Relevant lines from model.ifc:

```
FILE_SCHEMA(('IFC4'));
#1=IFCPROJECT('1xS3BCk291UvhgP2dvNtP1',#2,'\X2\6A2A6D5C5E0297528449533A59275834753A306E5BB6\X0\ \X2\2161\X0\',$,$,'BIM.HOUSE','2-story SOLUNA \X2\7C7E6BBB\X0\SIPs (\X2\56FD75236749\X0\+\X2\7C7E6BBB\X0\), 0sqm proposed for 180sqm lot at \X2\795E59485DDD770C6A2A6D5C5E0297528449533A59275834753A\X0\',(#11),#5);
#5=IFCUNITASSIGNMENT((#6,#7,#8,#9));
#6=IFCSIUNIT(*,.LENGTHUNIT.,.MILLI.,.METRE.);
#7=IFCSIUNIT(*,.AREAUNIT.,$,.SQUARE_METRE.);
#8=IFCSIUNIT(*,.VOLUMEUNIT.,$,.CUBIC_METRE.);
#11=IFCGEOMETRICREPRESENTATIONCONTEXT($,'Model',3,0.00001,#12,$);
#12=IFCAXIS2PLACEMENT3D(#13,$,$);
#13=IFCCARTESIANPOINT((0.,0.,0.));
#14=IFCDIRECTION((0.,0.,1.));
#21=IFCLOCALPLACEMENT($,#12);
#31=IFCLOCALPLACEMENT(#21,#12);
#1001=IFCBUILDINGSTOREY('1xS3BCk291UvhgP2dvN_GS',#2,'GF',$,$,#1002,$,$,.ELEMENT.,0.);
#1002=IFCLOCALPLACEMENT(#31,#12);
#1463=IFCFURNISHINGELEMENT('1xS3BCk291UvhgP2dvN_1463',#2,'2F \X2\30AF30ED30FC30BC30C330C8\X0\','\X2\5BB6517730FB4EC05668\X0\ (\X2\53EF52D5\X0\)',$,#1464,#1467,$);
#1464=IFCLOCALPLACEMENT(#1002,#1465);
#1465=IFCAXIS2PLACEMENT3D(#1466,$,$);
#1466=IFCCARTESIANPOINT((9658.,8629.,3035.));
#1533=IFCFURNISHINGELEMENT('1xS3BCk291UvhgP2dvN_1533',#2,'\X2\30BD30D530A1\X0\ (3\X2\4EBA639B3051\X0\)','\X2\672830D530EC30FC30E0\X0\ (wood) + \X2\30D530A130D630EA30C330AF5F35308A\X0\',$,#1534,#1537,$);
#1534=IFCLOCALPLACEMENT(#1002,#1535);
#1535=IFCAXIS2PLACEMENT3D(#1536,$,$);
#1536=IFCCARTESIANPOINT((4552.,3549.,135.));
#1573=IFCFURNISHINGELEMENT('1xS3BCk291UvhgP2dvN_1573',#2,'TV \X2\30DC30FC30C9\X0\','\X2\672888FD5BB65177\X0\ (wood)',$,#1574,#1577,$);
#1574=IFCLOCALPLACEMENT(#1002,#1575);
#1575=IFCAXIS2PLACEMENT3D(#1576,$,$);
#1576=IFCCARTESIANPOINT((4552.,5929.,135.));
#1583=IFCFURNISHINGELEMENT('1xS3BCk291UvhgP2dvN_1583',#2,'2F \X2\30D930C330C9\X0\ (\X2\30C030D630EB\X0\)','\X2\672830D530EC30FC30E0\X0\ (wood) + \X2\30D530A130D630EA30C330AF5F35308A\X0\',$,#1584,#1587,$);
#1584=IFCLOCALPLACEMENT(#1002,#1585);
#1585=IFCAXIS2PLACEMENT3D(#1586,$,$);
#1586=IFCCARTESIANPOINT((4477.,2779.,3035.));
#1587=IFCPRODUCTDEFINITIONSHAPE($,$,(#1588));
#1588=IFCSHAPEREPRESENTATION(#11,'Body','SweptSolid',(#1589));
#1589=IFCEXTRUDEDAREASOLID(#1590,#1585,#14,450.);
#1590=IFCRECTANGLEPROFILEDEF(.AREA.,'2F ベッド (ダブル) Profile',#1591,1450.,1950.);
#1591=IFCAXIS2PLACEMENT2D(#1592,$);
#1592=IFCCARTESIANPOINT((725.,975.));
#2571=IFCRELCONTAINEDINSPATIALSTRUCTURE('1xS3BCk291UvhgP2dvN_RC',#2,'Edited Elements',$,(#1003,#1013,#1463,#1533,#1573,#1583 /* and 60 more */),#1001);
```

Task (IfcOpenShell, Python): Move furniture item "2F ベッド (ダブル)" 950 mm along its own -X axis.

```python
import ifcopenshell
import ifcopenshell.api.geometry
import ifcopenshell.util.placement
import ifcopenshell.util.unit

model = ifcopenshell.open("model.ifc")
unit_scale = ifcopenshell.util.unit.calculate_unit_scale(model)

item = model.by_guid("1xS3BCk291UvhgP2dvN_1583")
matrix = ifcopenshell.util.placement.get_local_placement(item.ObjectPlacement)
matrix[:3, 3] -= matrix[:3, 0] * 0.95 / unit_scale
ifcopenshell.api.geometry.edit_object_placement(model, product=item, matrix=matrix, is_si=False)

print(ifcopenshell.util.placement.get_local_placement(item.ObjectPlacement).round(3) + 0.0)

model.write("model_rev.ifc")
```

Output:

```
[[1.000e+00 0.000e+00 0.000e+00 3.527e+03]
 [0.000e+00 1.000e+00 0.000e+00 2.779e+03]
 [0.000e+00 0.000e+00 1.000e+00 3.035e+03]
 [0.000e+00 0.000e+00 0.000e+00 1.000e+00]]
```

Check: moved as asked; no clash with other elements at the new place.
